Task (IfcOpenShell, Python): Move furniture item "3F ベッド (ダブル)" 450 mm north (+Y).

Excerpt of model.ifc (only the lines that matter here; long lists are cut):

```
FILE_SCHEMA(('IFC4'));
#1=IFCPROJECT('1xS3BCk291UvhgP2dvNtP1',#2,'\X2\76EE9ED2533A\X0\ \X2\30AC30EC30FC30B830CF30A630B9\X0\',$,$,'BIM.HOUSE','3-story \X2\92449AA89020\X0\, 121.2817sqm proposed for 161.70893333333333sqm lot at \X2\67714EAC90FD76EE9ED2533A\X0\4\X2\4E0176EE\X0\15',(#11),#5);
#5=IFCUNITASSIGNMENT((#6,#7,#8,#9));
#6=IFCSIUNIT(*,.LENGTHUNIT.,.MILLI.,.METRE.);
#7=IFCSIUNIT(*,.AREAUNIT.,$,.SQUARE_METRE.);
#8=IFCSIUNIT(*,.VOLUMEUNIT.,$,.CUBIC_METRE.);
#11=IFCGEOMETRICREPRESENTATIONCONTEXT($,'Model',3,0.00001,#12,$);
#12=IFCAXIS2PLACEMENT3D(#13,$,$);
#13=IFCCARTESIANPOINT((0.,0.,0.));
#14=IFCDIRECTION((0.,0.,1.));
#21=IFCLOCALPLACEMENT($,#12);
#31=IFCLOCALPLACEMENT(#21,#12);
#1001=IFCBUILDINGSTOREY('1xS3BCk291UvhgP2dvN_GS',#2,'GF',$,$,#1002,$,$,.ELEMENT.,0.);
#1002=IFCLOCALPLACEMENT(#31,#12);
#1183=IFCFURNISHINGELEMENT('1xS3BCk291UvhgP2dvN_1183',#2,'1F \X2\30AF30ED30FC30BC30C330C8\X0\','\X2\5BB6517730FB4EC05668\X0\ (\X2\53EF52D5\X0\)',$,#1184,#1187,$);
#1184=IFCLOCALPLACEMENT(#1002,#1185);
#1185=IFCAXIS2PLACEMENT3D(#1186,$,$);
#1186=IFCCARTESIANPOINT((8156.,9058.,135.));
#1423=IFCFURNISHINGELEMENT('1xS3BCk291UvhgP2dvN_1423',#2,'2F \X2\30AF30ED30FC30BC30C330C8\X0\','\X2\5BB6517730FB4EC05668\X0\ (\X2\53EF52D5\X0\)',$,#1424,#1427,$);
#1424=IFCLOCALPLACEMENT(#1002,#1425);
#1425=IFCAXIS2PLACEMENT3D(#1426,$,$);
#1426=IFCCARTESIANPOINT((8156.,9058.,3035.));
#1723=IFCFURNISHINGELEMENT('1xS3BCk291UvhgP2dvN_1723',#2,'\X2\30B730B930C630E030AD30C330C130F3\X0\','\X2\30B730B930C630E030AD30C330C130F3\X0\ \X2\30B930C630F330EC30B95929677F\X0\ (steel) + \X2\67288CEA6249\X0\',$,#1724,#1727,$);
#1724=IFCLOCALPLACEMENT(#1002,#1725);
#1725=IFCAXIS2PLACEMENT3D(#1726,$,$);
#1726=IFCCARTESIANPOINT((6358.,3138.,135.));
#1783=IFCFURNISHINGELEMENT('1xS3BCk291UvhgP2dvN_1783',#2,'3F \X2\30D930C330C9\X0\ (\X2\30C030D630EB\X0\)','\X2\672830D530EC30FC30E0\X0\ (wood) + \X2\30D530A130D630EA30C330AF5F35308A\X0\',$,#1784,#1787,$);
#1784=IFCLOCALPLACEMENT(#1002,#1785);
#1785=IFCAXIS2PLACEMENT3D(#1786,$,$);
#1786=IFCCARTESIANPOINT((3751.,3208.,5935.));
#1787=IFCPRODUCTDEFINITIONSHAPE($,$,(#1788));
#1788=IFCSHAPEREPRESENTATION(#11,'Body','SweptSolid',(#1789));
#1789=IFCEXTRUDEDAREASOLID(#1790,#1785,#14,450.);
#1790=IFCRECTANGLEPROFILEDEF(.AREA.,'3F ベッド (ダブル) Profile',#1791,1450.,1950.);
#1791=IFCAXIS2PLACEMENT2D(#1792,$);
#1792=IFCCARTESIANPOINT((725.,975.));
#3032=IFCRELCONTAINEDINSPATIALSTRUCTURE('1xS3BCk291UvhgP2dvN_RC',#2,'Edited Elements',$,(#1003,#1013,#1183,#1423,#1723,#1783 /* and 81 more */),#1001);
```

```python
import ifcopenshell
import ifcopenshell.api.geometry
import ifcopenshell.util.placement
import ifcopenshell.util.unit

model = ifcopenshell.open("model.ifc")
unit_scale = ifcopenshell.util.unit.calculate_unit_scale(model)

item = model.by_guid("1xS3BCk291UvhgP2dvN_1783")
matrix = ifcopenshell.util.placement.get_local_placement(item.ObjectPlacement)
matrix[1, 3] += 0.45 / unit_scale
ifcopenshell.api.geometry.edit_object_placement(model, product=item, matrix=matrix, is_si=False)

print(ifcopenshell.util.placement.get_local_placement(item.ObjectPlacement).round(3) + 0.0)

model.write("model_rev.ifc")
```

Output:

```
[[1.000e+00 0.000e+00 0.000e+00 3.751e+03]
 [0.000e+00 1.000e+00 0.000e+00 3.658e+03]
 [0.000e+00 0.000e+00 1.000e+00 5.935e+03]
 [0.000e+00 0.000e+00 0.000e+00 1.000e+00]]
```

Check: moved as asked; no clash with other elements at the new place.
